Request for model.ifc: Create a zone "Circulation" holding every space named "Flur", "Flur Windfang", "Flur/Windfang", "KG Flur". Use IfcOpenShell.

First a look at what the model holds.

```python
import ifcopenshell

model = ifcopenshell.open("model.ifc")
print(model.schema)
seen = {}
for space in model.by_type("IfcSpace"):
    seen[space.LongName] = seen.get(space.LongName, 0) + 1
for name, count in sorted(seen.items(), key=str):
    print(count, "x", name)
print("zones:", [z.Name for z in model.by_type("IfcZone")][:20])
```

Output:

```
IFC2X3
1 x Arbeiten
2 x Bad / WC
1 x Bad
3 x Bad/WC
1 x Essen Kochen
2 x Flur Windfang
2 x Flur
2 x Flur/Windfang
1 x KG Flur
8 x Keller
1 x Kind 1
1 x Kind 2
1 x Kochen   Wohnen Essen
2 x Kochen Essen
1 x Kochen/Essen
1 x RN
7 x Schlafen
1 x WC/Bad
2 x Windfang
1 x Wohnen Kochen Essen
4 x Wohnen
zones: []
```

```python
import ifcopenshell
import ifcopenshell.api.group
import ifcopenshell.api.root

model = ifcopenshell.open("model.ifc")

names = {"Flur", "Flur Windfang", "Flur/Windfang", "KG Flur"}
spaces = [s for s in model.by_type("IfcSpace") if s.LongName in names]

zone = ifcopenshell.api.root.create_entity(model, ifc_class="IfcZone", name="Circulation")
ifcopenshell.api.group.assign_group(model, products=spaces, group=zone)
print(len(spaces), "spaces in", zone.Name)

model.write("model_rev.ifc")
```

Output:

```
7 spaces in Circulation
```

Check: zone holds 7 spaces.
